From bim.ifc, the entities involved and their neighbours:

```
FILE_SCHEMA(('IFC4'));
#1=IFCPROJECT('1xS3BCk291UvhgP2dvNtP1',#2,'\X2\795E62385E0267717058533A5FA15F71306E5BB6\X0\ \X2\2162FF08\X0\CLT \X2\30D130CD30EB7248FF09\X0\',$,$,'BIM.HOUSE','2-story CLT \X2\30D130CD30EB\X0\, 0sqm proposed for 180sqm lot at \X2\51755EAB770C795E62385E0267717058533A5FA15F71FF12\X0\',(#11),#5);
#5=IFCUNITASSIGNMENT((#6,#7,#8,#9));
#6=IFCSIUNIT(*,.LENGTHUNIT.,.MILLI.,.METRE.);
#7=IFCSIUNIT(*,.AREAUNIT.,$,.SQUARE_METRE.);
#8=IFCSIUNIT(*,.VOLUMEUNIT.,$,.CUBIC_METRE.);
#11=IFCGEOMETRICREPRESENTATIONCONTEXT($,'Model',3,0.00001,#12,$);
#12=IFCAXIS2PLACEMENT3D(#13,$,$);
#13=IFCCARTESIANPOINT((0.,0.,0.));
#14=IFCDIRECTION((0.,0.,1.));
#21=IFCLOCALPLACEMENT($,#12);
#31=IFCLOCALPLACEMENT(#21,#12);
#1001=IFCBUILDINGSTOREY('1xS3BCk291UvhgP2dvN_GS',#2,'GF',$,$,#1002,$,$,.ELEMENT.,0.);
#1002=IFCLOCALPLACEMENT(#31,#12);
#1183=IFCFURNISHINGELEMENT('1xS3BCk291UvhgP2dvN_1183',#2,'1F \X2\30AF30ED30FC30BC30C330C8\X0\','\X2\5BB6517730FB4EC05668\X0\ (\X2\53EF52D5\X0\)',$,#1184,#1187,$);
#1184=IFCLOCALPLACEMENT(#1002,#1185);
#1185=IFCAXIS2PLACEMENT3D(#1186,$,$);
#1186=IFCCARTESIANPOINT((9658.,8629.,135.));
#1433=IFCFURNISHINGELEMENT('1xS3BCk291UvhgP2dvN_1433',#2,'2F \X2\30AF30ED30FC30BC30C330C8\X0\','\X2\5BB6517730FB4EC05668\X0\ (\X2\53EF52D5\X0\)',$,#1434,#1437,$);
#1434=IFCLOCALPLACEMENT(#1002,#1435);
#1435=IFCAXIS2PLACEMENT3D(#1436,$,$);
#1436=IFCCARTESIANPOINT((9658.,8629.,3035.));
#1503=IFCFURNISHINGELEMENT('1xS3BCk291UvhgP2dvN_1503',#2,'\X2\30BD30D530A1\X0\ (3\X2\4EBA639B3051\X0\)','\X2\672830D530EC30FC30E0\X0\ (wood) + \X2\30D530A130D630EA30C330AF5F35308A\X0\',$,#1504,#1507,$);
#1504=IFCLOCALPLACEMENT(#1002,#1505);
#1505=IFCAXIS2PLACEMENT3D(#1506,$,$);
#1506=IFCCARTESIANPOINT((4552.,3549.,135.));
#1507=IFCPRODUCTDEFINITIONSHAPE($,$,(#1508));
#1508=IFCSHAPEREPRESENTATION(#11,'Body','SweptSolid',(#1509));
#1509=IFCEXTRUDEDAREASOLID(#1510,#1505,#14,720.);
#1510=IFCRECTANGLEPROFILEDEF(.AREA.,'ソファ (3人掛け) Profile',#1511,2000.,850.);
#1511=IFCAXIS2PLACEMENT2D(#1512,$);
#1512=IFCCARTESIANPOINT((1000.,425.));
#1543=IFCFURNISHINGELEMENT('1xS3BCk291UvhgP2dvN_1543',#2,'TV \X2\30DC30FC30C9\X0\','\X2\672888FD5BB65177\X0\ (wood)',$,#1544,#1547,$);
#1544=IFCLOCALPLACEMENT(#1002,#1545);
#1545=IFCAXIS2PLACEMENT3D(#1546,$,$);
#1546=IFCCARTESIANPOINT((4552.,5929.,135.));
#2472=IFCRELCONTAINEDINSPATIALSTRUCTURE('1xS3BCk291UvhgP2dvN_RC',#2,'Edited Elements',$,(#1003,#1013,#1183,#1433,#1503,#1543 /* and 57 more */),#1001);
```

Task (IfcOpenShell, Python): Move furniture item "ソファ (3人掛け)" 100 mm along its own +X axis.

```python
import ifcopenshell
import ifcopenshell.api.geometry
import ifcopenshell.util.placement

model = ifcopenshell.open("bim.ifc")

item = model.by_guid("1xS3BCk291UvhgP2dvN_1503")
matrix = ifcopenshell.util.placement.get_local_placement(item.ObjectPlacement)
matrix[:3, 3] += matrix[:3, 0] * 100.0
ifcopenshell.api.geometry.edit_object_placement(model, product=item, matrix=matrix, is_si=False)

print(ifcopenshell.util.placement.get_local_placement(item.ObjectPlacement).round(3) + 0.0)

model.write("bim_v2.ifc")
```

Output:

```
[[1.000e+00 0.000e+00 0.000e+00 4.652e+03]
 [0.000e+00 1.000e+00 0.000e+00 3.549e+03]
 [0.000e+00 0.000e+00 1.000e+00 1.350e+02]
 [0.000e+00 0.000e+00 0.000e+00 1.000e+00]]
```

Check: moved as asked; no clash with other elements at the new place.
